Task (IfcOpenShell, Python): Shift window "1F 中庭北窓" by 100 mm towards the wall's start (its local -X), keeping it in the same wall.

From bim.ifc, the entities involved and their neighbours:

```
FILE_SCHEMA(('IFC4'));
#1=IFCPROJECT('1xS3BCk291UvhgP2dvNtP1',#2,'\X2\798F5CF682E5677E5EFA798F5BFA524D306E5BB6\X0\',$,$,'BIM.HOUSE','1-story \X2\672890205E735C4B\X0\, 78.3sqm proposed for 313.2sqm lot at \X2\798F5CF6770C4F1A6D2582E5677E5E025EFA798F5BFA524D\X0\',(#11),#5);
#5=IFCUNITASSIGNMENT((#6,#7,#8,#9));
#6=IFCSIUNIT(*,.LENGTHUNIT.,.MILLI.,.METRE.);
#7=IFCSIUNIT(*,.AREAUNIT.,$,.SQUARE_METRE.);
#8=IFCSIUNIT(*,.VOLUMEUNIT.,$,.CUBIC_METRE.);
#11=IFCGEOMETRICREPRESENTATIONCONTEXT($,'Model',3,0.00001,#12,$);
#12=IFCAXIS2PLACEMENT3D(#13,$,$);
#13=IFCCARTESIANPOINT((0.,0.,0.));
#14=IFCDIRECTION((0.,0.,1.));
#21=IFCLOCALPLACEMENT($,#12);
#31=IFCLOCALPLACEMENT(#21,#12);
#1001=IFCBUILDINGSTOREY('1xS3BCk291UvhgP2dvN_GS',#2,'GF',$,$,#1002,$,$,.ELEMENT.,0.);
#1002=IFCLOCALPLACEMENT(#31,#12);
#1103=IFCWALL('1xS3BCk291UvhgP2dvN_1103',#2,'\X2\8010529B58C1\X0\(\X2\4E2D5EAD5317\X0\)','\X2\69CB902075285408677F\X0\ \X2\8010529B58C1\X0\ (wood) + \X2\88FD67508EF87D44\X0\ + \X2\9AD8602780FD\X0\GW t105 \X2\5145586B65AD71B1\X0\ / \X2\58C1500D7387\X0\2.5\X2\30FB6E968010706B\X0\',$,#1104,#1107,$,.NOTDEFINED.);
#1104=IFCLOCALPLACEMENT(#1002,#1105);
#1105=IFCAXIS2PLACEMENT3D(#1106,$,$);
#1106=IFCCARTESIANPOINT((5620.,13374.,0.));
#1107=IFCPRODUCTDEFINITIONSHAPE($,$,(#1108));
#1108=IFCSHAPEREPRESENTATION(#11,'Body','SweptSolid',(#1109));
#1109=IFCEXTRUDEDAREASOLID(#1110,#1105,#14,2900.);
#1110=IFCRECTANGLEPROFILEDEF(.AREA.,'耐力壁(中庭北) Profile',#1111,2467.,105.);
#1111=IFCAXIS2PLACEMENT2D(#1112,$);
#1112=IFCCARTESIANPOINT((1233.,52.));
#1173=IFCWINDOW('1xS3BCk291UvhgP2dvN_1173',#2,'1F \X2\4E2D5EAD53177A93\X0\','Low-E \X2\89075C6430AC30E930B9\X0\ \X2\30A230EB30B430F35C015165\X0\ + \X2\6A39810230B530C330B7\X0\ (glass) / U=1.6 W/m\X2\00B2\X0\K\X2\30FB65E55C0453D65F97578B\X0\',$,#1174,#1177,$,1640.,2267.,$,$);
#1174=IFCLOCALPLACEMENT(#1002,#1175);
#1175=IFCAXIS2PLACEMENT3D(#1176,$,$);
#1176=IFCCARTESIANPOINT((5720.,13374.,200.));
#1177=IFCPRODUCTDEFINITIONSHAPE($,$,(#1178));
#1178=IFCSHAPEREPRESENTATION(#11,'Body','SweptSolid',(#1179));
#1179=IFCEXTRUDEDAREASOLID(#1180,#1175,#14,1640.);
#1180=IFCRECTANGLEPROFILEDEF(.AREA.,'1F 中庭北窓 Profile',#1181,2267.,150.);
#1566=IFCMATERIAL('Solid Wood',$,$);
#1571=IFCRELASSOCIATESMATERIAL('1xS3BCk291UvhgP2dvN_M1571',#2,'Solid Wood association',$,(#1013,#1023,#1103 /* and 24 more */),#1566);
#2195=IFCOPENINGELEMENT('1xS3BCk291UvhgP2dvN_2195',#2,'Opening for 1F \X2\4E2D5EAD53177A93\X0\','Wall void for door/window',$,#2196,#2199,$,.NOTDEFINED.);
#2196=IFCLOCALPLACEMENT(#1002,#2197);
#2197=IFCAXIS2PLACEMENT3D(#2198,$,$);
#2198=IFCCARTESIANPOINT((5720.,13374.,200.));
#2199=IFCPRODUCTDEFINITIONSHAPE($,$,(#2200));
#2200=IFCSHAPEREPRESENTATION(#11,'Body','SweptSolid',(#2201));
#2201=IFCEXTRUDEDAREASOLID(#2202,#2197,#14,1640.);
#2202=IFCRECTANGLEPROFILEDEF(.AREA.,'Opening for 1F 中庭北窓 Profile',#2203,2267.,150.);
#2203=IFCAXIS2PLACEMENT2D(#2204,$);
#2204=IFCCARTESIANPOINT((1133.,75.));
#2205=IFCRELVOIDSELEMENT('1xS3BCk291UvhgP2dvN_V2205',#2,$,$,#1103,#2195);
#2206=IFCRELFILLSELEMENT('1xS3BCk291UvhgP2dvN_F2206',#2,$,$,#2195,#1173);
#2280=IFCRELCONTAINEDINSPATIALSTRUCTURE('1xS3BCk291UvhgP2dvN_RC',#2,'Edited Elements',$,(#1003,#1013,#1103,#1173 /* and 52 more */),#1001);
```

```python
import ifcopenshell
import ifcopenshell.api.geometry
import ifcopenshell.util.placement

model = ifcopenshell.open("bim.ifc")

window = model.by_guid("1xS3BCk291UvhgP2dvN_1173")
opening = window.FillsVoids[0].RelatingOpeningElement
wall = opening.VoidsElements[0].RelatingBuildingElement

wall_matrix = ifcopenshell.util.placement.get_local_placement(wall.ObjectPlacement)
shift = wall_matrix[:3, 0] * -100.0
before = ifcopenshell.util.placement.get_local_placement(window.ObjectPlacement)[:3, 3].copy()

# The window is not placed relative to its opening, so move both.
for product in (opening, window):
    matrix = ifcopenshell.util.placement.get_local_placement(product.ObjectPlacement)
    matrix[:3, 3] += shift
    ifcopenshell.api.geometry.edit_object_placement(model, product=product, matrix=matrix, is_si=False)

after = ifcopenshell.util.placement.get_local_placement(window.ObjectPlacement)[:3, 3]
print("window moved by", (after - before).round(3) + 0.0)

model.write("bim_updated.ifc")
```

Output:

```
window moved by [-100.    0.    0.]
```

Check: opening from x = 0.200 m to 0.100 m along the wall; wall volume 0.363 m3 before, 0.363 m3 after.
